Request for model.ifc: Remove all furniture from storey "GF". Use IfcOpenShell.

First a look at what the model holds.

```python
import ifcopenshell
import ifcopenshell.util.element

model = ifcopenshell.open("model.ifc")
print(model.schema)
storey = next(s for s in model.by_type("IfcBuildingStorey") if s.Name == "GF")
furniture = [e for e in ifcopenshell.util.element.get_decomposition(storey) if e.is_a("IfcFurnishingElement")]
seen = {}
for e in furniture:
    element_type = ifcopenshell.util.element.get_type(e)
    name = element_type.Name if element_type not in (None, e) else None
    seen[name] = seen.get(name, 0) + 1
for name, count in sorted(seen.items(), key=str):
    print(count, "x", name)
```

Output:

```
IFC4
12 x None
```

```python
import ifcopenshell
import ifcopenshell.api.root
import ifcopenshell.util.element

model = ifcopenshell.open("model.ifc")

storey = next(s for s in model.by_type("IfcBuildingStorey") if s.Name == "GF")
furniture = [e for e in ifcopenshell.util.element.get_decomposition(storey) if e.is_a("IfcFurnishingElement")]

for e in furniture:
    ifcopenshell.api.root.remove_product(model, product=e)
print(len(furniture), "removed")

model.write("model_v2.ifc")
```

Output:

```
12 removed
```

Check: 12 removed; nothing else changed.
